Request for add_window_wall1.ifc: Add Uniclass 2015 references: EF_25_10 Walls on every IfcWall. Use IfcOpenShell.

First a look at what the model holds.

```python
import ifcopenshell

model = ifcopenshell.open("add_window_wall1.ifc")
print(model.schema)
print("classifications:", [c.Name for c in model.by_type("IfcClassification")])
for ifc_class in ("IfcDoor", "IfcRoof", "IfcStair", "IfcWall", "IfcWindow"):
    print(ifc_class, len(model.by_type(ifc_class)))
```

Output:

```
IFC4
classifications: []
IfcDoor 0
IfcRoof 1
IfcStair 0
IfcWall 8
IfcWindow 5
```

```python
import ifcopenshell
import ifcopenshell.api.classification

model = ifcopenshell.open("add_window_wall1.ifc")

system = ifcopenshell.api.classification.add_classification(model, classification="Uniclass 2015")

codes = {
    "IfcWall": ("EF_25_10", "Walls"),
}
for ifc_class, (code, name) in codes.items():
    products = model.by_type(ifc_class)
    ifcopenshell.api.classification.add_reference(
        model, products=products, classification=system, identification=code, name=name
    )
    print(code, len(products))

model.write("add_window_wall1_updated.ifc")
```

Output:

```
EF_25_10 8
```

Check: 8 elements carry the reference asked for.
